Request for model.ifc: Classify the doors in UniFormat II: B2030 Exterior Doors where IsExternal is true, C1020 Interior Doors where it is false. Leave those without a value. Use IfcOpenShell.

First a look at what the model holds.

```python
import ifcopenshell
import ifcopenshell.util.element

model = ifcopenshell.open("model.ifc")
print(model.schema)
print("classifications:", [c.Name for c in model.by_type("IfcClassification")])
values = [ifcopenshell.util.element.get_pset(e, "Pset_DoorCommon", "IsExternal") for e in model.by_type("IfcDoor")]
for value in (True, False, None):
    print("IsExternal", value, values.count(value))
```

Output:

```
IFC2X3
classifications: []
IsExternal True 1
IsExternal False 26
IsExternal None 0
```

```python
import ifcopenshell
import ifcopenshell.api.classification
import ifcopenshell.util.element

model = ifcopenshell.open("model.ifc")

# IFC2X3 requires Source and Edition and has no link from the project to the system.
system = model.create_entity("IfcClassification", Source="ASTM", Edition="E1557", Name="UniFormat II")

doors = model.by_type("IfcDoor")
external = {e: ifcopenshell.util.element.get_pset(e, "Pset_DoorCommon", "IsExternal") for e in doors}
for flag, code, name in ((True, "B2030", "Exterior Doors"), (False, "C1020", "Interior Doors")):
    products = [e for e in doors if external[e] is flag]
    ifcopenshell.api.classification.add_reference(
        model, products=products, classification=system, identification=code, name=name
    )
    print(code, len(products))

model.write("model_updated.ifc")
```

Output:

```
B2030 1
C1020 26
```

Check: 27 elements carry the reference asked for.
